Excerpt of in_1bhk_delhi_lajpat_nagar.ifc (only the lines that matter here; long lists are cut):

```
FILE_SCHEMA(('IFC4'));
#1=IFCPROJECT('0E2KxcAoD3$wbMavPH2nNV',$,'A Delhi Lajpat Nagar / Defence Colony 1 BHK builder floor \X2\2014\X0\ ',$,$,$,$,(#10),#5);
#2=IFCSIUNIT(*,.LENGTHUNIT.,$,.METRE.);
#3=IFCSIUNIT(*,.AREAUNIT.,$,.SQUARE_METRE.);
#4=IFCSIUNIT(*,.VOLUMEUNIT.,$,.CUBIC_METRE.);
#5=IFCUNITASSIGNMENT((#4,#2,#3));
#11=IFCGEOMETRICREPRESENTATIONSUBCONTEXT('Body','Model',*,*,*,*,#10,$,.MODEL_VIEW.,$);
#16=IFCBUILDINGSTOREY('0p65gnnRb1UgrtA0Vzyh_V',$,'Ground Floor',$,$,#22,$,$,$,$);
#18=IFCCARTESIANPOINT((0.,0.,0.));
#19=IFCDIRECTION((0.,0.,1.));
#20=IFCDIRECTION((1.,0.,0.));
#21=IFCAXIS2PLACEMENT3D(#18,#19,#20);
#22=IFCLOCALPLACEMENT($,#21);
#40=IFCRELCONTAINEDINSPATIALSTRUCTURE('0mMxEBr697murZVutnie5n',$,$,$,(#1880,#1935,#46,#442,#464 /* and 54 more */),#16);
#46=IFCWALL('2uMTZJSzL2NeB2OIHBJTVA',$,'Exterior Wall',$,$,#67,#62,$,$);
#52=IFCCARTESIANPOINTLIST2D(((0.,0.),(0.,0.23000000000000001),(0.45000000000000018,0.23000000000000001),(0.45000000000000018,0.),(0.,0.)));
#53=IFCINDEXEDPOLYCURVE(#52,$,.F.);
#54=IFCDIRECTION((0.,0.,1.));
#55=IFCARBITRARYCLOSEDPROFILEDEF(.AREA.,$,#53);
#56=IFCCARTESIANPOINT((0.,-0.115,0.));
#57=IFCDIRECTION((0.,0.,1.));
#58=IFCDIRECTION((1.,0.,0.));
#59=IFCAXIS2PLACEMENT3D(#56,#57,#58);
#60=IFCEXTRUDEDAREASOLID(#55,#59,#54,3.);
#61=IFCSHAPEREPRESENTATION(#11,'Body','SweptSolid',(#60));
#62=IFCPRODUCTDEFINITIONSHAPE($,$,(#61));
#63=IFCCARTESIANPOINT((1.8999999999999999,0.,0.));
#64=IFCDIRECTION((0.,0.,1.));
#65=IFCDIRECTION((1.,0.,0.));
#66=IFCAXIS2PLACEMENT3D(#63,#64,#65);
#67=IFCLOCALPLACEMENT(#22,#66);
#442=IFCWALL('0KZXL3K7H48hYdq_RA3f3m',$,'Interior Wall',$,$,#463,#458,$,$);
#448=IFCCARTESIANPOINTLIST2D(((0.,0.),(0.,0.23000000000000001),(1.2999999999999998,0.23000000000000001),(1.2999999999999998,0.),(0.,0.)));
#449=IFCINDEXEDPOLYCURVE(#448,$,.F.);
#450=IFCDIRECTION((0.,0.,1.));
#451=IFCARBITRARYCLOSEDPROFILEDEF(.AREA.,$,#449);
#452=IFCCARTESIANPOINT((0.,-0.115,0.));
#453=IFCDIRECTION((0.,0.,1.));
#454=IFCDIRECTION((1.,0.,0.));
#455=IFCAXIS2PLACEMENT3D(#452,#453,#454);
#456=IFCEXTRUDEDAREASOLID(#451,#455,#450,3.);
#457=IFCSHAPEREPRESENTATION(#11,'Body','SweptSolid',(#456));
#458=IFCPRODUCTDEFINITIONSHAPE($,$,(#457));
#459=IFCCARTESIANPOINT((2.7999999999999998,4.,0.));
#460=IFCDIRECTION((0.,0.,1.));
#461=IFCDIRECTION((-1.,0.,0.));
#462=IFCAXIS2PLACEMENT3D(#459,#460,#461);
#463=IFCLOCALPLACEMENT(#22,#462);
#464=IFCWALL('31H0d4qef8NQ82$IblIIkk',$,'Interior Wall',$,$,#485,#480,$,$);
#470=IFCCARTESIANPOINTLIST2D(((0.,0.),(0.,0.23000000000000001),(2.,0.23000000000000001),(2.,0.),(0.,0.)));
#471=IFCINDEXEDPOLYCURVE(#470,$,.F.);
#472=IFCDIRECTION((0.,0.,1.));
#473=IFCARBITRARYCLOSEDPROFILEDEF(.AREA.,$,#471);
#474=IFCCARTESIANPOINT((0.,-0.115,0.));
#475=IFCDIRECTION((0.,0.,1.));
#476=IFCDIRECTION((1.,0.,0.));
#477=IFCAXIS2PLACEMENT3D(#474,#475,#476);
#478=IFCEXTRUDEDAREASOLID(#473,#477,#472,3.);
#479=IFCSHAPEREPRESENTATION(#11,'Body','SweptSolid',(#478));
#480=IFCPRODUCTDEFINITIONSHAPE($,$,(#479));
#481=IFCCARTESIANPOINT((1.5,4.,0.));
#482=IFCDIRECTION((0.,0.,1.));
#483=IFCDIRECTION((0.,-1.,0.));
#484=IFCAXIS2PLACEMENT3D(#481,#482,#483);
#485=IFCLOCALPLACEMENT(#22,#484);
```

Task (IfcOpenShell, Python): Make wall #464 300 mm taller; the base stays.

```python
import ifcopenshell
import ifcopenshell.geom
import ifcopenshell.util.representation
import ifcopenshell.util.shape
import ifcopenshell.util.unit

model = ifcopenshell.open("in_1bhk_delhi_lajpat_nagar.ifc")
unit_scale = ifcopenshell.util.unit.calculate_unit_scale(model)
settings = ifcopenshell.geom.settings()


def volume(element):
    """Net volume in cubic metres, openings subtracted."""
    shape = ifcopenshell.geom.create_shape(settings, element)
    return ifcopenshell.util.shape.get_volume(shape.geometry)


wall = model.by_guid("31H0d4qef8NQ82$IblIIkk")
before = volume(wall)

body = ifcopenshell.util.representation.get_representation(wall, "Model", "Body")
solid = body.Items[0]
old_height = solid.Depth
solid.Depth += 0.3 / unit_scale
after = volume(wall)

print(f"height {old_height:g} -> {solid.Depth:g}, volume {before:.3f} -> {after:.3f} m3")

model.write("in_1bhk_delhi_lajpat_nagar_v2.ifc")
```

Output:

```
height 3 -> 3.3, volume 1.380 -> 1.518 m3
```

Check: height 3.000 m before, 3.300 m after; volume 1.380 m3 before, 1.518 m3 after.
